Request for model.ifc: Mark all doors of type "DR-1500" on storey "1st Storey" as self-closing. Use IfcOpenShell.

First a look at what the model holds.

```python
import ifcopenshell
import ifcopenshell.util.element

model = ifcopenshell.open("model.ifc")
print(model.schema)
storey = next(s for s in model.by_type("IfcBuildingStorey") if s.Name == "1st Storey")
doors = [e for e in ifcopenshell.util.element.get_decomposition(storey) if e.is_a("IfcDoor")]
seen = {}
for e in doors:
    element_type = ifcopenshell.util.element.get_type(e)
    key = (element_type.Name if element_type != e and element_type else None, ifcopenshell.util.element.get_pset(e, "Pset_DoorCommon", "SelfClosing"))
    seen[key] = seen.get(key, 0) + 1
for (name, value), count in sorted(seen.items(), key=str):
    print(count, "x", name, "|", value)
```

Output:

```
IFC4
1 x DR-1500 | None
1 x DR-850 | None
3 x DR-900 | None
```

```python
import ifcopenshell
import ifcopenshell.api.pset
import ifcopenshell.util.element

model = ifcopenshell.open("model.ifc")

storey = next(s for s in model.by_type("IfcBuildingStorey") if s.Name == "1st Storey")
doors = [e for e in ifcopenshell.util.element.get_decomposition(storey) if e.is_a("IfcDoor")]

count = 0
for e in doors:
    element_type = ifcopenshell.util.element.get_type(e)
    if element_type in (None, e) or element_type.Name != "DR-1500":
        continue
    # add_pset returns the element's existing set when there is one.
    pset = ifcopenshell.api.pset.add_pset(model, product=e, name="Pset_DoorCommon")
    ifcopenshell.api.pset.edit_pset(model, pset=pset, properties={"SelfClosing": True})
    count += 1

print(count, "doors updated")

model.write("model_edited.ifc")
```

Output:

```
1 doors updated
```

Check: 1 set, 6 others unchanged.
